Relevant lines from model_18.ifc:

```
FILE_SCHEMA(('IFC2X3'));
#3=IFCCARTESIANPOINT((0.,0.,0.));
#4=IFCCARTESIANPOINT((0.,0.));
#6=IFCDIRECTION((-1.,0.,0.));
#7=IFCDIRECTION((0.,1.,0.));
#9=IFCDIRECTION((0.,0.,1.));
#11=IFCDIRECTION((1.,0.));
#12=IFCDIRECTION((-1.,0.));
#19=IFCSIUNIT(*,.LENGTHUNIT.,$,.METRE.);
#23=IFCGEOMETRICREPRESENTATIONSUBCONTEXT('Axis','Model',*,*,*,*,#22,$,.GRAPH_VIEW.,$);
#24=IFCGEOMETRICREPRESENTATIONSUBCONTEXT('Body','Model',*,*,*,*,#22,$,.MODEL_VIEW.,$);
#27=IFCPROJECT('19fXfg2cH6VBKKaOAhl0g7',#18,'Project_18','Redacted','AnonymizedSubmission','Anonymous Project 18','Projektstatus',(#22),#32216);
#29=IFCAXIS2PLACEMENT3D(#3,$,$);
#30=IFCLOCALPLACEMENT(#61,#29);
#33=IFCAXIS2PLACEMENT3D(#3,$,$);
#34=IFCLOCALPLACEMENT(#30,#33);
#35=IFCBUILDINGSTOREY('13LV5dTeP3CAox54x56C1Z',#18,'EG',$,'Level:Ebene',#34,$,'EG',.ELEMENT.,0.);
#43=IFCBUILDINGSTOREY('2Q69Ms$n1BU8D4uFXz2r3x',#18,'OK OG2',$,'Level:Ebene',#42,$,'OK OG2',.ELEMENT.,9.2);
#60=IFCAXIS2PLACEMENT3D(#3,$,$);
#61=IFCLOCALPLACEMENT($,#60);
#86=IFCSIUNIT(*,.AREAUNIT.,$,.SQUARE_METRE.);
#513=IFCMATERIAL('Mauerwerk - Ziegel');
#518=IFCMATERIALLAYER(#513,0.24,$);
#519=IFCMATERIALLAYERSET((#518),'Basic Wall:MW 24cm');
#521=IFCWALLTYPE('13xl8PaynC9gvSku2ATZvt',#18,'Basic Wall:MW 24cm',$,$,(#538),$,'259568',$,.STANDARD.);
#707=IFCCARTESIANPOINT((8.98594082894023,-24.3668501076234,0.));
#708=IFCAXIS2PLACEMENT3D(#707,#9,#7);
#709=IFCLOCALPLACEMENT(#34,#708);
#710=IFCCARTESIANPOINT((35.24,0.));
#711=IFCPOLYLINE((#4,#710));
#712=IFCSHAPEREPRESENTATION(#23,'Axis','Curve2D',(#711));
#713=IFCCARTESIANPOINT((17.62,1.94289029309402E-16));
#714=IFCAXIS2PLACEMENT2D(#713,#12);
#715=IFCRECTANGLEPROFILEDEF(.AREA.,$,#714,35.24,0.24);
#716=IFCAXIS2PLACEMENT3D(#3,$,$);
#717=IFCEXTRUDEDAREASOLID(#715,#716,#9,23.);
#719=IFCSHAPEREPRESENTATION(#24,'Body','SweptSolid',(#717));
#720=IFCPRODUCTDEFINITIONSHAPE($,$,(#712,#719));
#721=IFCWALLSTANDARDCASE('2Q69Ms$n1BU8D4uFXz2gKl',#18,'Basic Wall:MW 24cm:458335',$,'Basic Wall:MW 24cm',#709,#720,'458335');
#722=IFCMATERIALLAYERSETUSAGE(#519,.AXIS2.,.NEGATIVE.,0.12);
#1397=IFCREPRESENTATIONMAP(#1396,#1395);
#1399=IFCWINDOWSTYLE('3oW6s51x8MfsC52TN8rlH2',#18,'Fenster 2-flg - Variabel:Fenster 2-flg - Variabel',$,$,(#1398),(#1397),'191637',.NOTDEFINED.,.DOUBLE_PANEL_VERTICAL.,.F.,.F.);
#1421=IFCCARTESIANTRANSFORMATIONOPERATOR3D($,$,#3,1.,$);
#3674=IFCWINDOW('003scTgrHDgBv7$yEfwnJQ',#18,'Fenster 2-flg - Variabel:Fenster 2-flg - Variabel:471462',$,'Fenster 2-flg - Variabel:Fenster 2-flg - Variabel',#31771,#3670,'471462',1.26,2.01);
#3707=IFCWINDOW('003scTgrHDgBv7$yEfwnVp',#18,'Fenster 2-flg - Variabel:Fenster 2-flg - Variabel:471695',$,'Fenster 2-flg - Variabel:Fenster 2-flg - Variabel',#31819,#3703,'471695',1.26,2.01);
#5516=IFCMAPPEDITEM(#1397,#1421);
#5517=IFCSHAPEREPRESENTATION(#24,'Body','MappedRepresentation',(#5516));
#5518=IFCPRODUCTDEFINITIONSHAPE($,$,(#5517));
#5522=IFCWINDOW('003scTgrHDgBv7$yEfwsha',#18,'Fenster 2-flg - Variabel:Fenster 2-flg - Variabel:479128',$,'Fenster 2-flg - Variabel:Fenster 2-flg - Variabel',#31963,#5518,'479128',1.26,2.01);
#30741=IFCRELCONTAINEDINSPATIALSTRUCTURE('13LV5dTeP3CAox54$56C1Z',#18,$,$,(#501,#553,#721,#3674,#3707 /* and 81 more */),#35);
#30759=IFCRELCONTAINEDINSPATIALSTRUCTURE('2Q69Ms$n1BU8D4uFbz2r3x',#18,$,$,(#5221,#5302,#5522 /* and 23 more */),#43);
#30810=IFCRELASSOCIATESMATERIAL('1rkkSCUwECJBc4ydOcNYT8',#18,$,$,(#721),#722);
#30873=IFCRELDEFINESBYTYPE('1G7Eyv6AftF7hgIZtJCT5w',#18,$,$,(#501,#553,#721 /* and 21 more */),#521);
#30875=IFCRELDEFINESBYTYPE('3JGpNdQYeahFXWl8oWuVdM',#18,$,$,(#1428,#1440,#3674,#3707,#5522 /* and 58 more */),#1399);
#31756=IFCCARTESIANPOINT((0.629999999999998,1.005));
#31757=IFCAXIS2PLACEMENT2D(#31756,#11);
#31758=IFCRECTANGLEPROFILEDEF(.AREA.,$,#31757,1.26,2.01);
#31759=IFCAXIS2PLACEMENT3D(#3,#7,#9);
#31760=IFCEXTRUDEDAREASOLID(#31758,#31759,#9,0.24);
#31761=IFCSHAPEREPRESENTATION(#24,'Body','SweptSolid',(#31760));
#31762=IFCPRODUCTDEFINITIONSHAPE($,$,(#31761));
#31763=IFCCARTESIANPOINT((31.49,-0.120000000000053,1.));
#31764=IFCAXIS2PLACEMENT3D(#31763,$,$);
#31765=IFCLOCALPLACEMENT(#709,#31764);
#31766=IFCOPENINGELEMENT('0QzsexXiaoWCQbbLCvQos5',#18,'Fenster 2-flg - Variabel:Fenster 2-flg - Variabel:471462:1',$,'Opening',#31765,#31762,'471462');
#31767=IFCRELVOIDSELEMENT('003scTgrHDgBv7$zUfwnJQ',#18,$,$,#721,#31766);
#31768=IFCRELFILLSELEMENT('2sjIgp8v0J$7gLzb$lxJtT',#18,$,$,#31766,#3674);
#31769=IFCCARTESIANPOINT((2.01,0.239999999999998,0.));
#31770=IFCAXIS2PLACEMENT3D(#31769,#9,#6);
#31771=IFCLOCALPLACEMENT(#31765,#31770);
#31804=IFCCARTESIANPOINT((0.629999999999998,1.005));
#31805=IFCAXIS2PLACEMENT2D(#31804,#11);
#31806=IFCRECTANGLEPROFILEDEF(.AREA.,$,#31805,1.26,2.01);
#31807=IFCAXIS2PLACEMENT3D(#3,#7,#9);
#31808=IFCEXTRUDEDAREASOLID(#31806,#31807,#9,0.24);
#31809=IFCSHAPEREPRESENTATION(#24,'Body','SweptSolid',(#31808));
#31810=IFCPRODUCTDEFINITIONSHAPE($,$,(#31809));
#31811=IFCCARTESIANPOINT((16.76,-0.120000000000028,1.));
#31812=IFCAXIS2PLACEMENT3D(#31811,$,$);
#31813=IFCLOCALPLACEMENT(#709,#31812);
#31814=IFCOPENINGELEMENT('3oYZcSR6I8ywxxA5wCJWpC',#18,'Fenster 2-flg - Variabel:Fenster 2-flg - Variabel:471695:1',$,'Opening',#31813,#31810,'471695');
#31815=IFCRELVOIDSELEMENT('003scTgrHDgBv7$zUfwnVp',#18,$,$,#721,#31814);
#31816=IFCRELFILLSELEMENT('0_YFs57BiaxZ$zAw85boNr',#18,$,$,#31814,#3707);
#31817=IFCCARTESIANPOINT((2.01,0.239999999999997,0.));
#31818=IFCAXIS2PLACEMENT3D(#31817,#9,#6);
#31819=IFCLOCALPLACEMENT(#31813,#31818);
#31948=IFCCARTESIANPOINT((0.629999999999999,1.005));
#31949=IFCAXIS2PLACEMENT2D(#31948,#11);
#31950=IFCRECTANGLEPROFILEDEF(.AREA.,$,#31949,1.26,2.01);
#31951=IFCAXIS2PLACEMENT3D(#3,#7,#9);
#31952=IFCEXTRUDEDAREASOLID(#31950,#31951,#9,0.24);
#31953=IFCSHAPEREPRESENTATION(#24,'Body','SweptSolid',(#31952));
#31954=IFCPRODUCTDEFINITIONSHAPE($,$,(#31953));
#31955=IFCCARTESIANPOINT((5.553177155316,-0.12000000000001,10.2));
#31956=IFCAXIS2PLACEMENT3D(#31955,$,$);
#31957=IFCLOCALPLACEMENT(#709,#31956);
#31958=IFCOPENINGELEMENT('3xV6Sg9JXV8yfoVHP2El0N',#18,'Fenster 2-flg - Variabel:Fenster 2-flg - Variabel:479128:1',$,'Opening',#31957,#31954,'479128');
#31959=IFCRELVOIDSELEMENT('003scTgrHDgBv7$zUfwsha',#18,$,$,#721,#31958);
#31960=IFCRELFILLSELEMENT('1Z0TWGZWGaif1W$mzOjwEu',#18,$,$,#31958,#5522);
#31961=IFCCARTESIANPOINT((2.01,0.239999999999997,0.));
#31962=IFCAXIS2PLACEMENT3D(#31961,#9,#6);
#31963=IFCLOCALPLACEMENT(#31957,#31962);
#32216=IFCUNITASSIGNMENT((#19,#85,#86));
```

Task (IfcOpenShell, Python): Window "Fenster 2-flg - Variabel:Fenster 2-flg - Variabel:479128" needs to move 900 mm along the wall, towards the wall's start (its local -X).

```python
import ifcopenshell
import ifcopenshell.api.geometry
import ifcopenshell.util.placement

model = ifcopenshell.open("model_18.ifc")

window = model.by_guid("003scTgrHDgBv7$yEfwsha")
opening = window.FillsVoids[0].RelatingOpeningElement
wall = opening.VoidsElements[0].RelatingBuildingElement

wall_matrix = ifcopenshell.util.placement.get_local_placement(wall.ObjectPlacement)
shift = wall_matrix[:3, 0] * -0.9
before = ifcopenshell.util.placement.get_local_placement(window.ObjectPlacement)[:3, 3].copy()

# The window is placed relative to its opening, so it follows when the opening moves.
matrix = ifcopenshell.util.placement.get_local_placement(opening.ObjectPlacement)
matrix[:3, 3] += shift
ifcopenshell.api.geometry.edit_object_placement(
    model, product=opening, matrix=matrix, is_si=False, should_transform_children=True
)

after = ifcopenshell.util.placement.get_local_placement(window.ObjectPlacement)[:3, 3]
print("window moved by", (after - before).round(3) + 0.0)

model.write("model_18_updated.ifc")
```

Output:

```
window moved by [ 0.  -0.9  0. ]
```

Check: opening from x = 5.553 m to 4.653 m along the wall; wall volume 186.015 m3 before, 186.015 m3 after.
